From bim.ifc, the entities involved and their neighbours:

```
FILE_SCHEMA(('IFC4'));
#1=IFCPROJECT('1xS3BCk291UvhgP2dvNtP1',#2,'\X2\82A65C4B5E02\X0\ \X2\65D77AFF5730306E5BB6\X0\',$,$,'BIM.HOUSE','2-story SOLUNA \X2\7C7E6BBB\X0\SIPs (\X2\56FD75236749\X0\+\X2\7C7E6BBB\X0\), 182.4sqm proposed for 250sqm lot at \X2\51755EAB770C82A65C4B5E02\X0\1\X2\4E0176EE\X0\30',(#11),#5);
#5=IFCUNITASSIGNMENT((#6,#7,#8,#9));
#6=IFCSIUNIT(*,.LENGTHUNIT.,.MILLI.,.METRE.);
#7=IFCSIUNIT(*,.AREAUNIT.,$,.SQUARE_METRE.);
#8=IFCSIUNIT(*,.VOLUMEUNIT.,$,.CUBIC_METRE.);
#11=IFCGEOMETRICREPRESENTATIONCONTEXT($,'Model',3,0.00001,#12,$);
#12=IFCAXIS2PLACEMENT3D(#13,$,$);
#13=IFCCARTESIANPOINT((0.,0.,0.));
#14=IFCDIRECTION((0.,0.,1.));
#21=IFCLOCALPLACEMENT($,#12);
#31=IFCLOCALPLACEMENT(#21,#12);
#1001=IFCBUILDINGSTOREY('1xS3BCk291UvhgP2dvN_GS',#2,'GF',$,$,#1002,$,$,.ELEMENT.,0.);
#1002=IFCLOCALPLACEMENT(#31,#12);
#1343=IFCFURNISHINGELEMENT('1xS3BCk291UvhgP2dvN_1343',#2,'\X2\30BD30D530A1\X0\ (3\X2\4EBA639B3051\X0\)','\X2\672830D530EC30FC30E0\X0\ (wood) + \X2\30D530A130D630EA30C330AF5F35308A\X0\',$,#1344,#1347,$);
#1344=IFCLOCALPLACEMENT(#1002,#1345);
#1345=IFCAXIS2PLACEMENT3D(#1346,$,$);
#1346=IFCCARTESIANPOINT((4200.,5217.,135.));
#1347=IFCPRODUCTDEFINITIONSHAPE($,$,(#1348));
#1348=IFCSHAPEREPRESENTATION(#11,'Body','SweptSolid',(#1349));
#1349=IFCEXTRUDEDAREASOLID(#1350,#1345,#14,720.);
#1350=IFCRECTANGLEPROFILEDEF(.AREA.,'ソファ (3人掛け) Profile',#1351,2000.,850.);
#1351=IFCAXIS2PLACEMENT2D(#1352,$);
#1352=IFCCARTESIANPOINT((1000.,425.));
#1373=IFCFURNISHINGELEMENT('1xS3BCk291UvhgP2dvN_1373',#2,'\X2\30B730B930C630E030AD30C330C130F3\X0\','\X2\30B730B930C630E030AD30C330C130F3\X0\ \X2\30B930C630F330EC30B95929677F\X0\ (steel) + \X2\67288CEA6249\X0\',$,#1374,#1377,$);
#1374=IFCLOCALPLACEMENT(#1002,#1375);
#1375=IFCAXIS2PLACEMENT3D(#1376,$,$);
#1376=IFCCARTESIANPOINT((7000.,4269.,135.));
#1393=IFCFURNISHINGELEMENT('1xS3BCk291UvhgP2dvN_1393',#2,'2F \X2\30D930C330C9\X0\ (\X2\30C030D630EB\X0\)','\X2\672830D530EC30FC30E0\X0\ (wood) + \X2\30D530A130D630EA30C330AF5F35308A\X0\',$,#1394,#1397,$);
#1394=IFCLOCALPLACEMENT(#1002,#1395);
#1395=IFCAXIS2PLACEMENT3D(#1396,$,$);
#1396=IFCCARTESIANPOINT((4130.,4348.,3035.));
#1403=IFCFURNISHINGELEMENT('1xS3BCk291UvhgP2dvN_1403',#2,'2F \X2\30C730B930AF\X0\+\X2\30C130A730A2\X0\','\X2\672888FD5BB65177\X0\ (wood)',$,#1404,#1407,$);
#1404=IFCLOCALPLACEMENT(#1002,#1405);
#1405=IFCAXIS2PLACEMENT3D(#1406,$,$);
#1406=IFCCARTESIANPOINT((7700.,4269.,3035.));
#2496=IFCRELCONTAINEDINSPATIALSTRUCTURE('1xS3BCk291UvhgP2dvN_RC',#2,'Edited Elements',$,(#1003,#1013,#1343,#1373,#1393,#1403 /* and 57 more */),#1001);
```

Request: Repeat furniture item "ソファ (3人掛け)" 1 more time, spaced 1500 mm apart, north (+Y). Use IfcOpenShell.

```python
import numpy as np
import ifcopenshell
import ifcopenshell.api.geometry
import ifcopenshell.api.root
import ifcopenshell.util.element
import ifcopenshell.util.placement
import ifcopenshell.util.unit

model = ifcopenshell.open("bim.ifc")
unit_scale = ifcopenshell.util.unit.calculate_unit_scale(model)


def reuse_history(source, copy):
    """copy_class also copies each property set's owner history, people and application; keep the originals."""
    for rel in copy.IsDefinedBy:
        if rel.is_a("IfcRelDefinesByProperties") and (history := rel.RelatingPropertyDefinition.OwnerHistory):
            rel.RelatingPropertyDefinition.OwnerHistory = source.OwnerHistory
            ifcopenshell.util.element.remove_deep2(model, history)


source = model.by_guid("1xS3BCk291UvhgP2dvN_1343")
base = ifcopenshell.util.placement.get_local_placement(source.ObjectPlacement)
step = np.array([0.0, 1.0, 0.0]) * 1.5 / unit_scale

for i in range(1, 2):
    copy = ifcopenshell.api.root.copy_class(model, product=source)
    copy.Representation = ifcopenshell.util.element.copy_deep(
        model, source.Representation, exclude=["IfcGeometricRepresentationContext", "IfcRepresentationMap"]
    )
    reuse_history(source, copy)
    matrix = base.copy()
    matrix[:3, 3] += i * step
    print("added at", matrix[:3, 3].round(3) + 0.0)
    ifcopenshell.api.geometry.edit_object_placement(model, product=copy, matrix=matrix, is_si=False)

model.write("bim_rev.ifc")
```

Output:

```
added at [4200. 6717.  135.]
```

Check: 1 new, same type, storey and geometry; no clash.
